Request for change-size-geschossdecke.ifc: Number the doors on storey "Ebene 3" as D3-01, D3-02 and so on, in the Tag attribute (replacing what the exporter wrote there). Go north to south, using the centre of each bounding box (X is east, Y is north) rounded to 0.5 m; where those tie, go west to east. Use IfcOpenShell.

First a look at what the model holds.

```python
import ifcopenshell
import ifcopenshell.util.element
import ifcopenshell.util.placement

model = ifcopenshell.open("change-size-geschossdecke.ifc")
print(model.schema)
storey = next(s for s in model.by_type("IfcBuildingStorey") if s.Name == "Ebene 3")
doors = [e for e in ifcopenshell.util.element.get_decomposition(storey) if e.is_a("IfcDoor")]
for e in sorted(doors, key=lambda e: e.id()):
    origin = ifcopenshell.util.placement.get_local_placement(e.ObjectPlacement)[:3, 3]
    print(e.id(), e.Tag, e.Name, origin.round(2) + 0.0, sep=" | ")
```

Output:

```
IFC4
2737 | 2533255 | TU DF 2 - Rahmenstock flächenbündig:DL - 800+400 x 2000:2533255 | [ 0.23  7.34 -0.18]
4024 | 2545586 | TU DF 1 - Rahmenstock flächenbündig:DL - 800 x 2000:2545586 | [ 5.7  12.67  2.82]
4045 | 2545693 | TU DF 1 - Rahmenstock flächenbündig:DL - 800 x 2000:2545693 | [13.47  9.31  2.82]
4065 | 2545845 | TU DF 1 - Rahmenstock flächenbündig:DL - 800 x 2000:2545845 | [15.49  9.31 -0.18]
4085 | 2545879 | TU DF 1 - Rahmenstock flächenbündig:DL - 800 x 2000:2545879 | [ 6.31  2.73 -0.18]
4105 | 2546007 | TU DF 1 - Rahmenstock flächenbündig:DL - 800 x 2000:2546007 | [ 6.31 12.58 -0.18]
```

```python
import ifcopenshell
import ifcopenshell.geom
import ifcopenshell.util.element
import ifcopenshell.util.shape

model = ifcopenshell.open("change-size-geschossdecke.ifc")
settings = ifcopenshell.geom.settings()
settings.set("use-world-coords", True)


def centre(element):
    shape = ifcopenshell.geom.create_shape(settings, element)
    return ifcopenshell.util.shape.get_bbox_centroid(shape.geometry)


storey = next(s for s in model.by_type("IfcBuildingStorey") if s.Name == "Ebene 3")
doors = [e for e in ifcopenshell.util.element.get_decomposition(storey) if e.is_a("IfcDoor")]

# Insertion points can sit at a corner or the storey origin, so sort by the geometry (in metres).
centres = {e: centre(e) for e in doors}
doors.sort(key=lambda e: (-round(centres[e][1] / 0.5), centres[e][0]))

for i, e in enumerate(doors, start=1):
    number = f"D3-{i:02d}"
    e.Tag = number
    print(e.id(), number)

model.write("change-size-geschossdecke_v2.ifc")
```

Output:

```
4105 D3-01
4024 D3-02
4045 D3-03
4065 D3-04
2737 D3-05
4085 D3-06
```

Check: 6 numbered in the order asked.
